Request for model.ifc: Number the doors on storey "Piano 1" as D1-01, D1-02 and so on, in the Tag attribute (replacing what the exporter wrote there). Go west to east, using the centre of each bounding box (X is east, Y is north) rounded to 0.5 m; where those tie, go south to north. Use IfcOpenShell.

First a look at what the model holds.

```python
import ifcopenshell
import ifcopenshell.util.element
import ifcopenshell.util.placement

model = ifcopenshell.open("model.ifc")
print(model.schema)
storey = next(s for s in model.by_type("IfcBuildingStorey") if s.Name == "Piano 1")
doors = [e for e in ifcopenshell.util.element.get_decomposition(storey) if e.is_a("IfcDoor")]
for e in sorted(doors, key=lambda e: e.id()):
    origin = ifcopenshell.util.placement.get_local_placement(e.ObjectPlacement)[:3, 3]
    print(e.id(), e.Tag, e.Name, origin.round(2) + 0.0, sep=" | ")
```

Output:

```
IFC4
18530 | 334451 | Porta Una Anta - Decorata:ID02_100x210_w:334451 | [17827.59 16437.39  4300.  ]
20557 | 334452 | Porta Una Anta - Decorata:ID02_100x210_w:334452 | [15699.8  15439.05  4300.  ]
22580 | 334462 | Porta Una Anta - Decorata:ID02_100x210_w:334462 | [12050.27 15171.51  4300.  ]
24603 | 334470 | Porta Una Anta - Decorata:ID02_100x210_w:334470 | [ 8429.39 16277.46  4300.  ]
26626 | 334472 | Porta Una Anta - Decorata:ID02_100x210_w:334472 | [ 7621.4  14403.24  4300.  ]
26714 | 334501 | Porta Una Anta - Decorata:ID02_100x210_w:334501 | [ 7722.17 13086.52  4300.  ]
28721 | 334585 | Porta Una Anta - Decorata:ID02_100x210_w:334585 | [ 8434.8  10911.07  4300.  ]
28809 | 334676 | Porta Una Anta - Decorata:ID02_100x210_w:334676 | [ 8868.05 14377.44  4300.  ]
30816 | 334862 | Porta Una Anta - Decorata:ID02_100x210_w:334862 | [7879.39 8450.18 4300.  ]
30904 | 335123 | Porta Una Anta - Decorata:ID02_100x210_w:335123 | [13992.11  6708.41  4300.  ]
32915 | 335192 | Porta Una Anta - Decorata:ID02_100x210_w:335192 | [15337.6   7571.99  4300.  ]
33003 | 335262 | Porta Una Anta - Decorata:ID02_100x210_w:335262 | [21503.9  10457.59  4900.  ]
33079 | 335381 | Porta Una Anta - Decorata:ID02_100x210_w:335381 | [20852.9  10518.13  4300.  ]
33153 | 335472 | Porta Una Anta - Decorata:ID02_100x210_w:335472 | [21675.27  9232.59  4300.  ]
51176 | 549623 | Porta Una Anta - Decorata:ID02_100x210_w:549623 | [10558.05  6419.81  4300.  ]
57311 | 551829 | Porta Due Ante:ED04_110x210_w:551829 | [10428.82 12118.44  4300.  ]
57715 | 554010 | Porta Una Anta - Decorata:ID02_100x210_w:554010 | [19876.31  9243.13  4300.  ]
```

```python
import ifcopenshell
import ifcopenshell.geom
import ifcopenshell.util.element
import ifcopenshell.util.shape

model = ifcopenshell.open("model.ifc")
settings = ifcopenshell.geom.settings()
settings.set("use-world-coords", True)


def centre(element):
    shape = ifcopenshell.geom.create_shape(settings, element)
    return ifcopenshell.util.shape.get_bbox_centroid(shape.geometry)


storey = next(s for s in model.by_type("IfcBuildingStorey") if s.Name == "Piano 1")
doors = [e for e in ifcopenshell.util.element.get_decomposition(storey) if e.is_a("IfcDoor")]

# Insertion points can sit at a corner or the storey origin, so sort by the geometry (in metres).
centres = {e: centre(e) for e in doors}
doors.sort(key=lambda e: (round(centres[e][0] / 0.5), centres[e][1]))

for i, e in enumerate(doors, start=1):
    number = f"D1-{i:02d}"
    e.Tag = number
    print(e.id(), number)

model.write("model-out.ifc")
```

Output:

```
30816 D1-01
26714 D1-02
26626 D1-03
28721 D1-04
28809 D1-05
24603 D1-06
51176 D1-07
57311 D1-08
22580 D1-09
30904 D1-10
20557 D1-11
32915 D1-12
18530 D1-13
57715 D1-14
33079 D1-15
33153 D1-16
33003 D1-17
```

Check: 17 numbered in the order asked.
